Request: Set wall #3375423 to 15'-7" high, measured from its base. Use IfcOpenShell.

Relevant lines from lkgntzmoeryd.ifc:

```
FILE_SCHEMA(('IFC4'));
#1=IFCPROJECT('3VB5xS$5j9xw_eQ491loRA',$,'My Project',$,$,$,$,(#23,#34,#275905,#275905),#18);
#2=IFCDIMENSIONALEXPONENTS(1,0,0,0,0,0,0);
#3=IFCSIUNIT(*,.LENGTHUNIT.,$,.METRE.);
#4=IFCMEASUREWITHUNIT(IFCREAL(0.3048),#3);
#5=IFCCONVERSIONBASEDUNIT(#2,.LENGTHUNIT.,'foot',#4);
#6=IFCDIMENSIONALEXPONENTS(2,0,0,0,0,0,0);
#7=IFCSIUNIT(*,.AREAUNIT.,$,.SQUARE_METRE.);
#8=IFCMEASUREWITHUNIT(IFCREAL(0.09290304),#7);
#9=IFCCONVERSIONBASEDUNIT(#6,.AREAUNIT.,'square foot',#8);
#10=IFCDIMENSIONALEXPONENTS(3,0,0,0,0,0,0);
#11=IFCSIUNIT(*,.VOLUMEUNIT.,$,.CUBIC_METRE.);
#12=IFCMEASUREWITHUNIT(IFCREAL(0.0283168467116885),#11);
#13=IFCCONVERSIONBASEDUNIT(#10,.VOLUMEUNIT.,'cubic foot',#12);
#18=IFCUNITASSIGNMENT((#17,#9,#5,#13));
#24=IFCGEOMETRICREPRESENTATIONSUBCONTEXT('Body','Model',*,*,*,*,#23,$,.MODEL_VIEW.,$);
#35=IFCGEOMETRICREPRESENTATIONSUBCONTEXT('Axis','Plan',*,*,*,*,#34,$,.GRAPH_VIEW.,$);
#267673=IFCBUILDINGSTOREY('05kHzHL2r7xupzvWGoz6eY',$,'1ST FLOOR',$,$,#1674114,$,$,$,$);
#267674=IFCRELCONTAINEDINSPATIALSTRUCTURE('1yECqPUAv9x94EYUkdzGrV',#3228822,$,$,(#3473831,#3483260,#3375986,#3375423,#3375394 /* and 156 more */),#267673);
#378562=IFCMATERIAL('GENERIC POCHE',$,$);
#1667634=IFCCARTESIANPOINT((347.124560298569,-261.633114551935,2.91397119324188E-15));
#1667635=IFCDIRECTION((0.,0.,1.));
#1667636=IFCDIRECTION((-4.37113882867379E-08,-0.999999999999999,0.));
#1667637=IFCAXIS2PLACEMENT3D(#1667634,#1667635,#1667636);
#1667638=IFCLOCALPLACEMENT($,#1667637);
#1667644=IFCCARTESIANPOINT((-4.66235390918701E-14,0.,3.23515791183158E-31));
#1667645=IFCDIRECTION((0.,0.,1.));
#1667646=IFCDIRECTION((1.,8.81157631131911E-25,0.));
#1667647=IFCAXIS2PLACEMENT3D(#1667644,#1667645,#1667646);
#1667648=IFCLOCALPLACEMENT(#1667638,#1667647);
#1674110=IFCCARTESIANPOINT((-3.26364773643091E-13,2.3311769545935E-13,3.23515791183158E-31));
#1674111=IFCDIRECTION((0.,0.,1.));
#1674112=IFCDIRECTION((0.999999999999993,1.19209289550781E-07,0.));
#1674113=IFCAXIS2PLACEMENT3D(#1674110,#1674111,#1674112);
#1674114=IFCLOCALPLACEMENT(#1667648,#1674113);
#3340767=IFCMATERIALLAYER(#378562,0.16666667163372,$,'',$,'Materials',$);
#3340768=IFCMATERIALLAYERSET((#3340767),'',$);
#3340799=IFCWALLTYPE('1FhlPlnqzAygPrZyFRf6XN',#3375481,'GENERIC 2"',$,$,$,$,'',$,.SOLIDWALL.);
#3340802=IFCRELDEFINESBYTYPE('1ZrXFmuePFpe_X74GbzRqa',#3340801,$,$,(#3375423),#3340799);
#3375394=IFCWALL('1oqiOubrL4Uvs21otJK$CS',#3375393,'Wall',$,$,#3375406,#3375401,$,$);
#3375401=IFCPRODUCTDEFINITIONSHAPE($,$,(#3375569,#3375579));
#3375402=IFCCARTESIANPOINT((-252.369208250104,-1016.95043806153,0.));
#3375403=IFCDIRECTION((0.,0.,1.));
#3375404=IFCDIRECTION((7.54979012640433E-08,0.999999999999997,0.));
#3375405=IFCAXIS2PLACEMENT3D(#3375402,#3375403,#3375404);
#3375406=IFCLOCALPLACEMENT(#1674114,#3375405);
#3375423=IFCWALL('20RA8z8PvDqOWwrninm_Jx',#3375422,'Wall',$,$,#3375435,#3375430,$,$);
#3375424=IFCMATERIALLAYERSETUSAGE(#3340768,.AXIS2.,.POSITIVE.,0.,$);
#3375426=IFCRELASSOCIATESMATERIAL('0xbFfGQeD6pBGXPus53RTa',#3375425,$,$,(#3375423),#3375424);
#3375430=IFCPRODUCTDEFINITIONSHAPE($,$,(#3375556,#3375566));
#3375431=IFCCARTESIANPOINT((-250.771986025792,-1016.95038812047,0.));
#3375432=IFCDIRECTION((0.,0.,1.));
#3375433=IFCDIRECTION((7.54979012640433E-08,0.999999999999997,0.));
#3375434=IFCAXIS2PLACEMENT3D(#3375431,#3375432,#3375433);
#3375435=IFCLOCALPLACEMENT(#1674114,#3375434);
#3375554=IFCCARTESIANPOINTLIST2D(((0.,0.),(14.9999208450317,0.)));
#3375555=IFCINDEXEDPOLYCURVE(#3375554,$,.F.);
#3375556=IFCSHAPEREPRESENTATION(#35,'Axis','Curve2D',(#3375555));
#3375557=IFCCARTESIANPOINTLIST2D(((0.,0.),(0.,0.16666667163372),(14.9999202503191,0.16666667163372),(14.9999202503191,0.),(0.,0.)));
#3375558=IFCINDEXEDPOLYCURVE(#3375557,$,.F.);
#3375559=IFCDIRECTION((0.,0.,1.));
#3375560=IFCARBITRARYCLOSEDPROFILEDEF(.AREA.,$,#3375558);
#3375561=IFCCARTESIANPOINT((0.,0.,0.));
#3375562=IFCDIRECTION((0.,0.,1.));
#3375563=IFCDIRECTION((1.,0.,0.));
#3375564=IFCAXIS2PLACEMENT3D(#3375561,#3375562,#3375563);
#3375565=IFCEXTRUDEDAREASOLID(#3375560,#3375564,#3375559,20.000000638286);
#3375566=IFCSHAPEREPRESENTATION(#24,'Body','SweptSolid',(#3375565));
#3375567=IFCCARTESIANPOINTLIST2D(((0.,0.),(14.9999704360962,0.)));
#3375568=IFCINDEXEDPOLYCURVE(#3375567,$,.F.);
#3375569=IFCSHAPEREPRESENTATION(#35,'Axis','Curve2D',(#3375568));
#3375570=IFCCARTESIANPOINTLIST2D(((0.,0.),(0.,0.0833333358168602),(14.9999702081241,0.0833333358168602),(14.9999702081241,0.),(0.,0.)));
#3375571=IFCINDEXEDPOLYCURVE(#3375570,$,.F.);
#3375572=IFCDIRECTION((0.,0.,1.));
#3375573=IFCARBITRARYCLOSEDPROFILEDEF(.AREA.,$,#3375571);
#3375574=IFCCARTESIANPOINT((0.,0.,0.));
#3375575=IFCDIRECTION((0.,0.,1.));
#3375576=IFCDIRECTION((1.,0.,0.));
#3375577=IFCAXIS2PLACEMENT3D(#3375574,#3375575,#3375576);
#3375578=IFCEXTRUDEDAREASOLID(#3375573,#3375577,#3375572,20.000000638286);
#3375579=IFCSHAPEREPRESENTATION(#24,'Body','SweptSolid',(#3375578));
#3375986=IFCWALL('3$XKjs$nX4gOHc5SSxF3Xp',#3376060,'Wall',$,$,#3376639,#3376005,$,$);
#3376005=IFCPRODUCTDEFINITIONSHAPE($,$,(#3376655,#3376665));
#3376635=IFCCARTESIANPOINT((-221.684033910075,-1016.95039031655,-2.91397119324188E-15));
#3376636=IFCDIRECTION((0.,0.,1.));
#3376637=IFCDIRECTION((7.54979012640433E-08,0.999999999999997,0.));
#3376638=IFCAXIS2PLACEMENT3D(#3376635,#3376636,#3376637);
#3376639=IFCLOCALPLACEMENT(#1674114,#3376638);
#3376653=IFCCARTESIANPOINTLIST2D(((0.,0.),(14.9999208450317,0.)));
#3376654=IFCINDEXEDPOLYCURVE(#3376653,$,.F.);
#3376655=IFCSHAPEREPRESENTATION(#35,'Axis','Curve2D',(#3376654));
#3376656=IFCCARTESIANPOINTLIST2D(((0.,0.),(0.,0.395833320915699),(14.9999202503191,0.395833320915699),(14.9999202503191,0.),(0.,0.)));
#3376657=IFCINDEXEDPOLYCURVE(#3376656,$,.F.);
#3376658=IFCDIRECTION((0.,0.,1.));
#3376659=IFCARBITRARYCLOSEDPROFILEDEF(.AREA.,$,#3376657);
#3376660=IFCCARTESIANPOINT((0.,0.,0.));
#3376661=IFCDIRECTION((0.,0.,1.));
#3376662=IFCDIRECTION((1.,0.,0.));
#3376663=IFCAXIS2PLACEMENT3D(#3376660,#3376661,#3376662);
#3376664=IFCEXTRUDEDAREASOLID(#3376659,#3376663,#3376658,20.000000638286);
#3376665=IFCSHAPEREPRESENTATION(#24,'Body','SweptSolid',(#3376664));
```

```python
import ifcopenshell
import ifcopenshell.geom
import ifcopenshell.util.representation
import ifcopenshell.util.shape
import ifcopenshell.util.unit

model = ifcopenshell.open("lkgntzmoeryd.ifc")
unit_scale = ifcopenshell.util.unit.calculate_unit_scale(model)
settings = ifcopenshell.geom.settings()


def volume(element):
    """Net volume in cubic metres, openings subtracted."""
    shape = ifcopenshell.geom.create_shape(settings, element)
    return ifcopenshell.util.shape.get_volume(shape.geometry)


wall = model.by_id(3375423)
before = volume(wall)

body = ifcopenshell.util.representation.get_representation(wall, "Model", "Body")
solid = body.Items[0]
old_height = solid.Depth
solid.Depth = 187 * 0.0254 / unit_scale
after = volume(wall)

print(f"height {old_height:g} -> {solid.Depth:g}, volume {before:.3f} -> {after:.3f} m3")

model.write("lkgntzmoeryd_updated.ifc")
```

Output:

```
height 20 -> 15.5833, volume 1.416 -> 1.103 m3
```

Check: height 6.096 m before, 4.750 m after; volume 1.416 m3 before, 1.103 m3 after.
